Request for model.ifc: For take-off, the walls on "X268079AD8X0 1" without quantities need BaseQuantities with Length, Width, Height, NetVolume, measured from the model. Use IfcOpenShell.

First a look at what the model holds.

```python
import ifcopenshell
import ifcopenshell.util.element
import ifcopenshell.util.unit

model = ifcopenshell.open("model.ifc")
print(model.schema)
for unit_type in ("LENGTHUNIT", "AREAUNIT", "VOLUMEUNIT"):
    print(unit_type, ifcopenshell.util.unit.calculate_unit_scale(model, unit_type))
storey = next(s for s in model.by_type("IfcBuildingStorey") if s.Name == "X268079AD8X0 1")
walls = [e for e in ifcopenshell.util.element.get_decomposition(storey) if e.is_a("IfcWall")]
for e in sorted(walls, key=lambda e: e.id()):
    print(e.id(), e.is_a(), e.Name, list(ifcopenshell.util.element.get_psets(e, qtos_only=True)), sep=" | ")
```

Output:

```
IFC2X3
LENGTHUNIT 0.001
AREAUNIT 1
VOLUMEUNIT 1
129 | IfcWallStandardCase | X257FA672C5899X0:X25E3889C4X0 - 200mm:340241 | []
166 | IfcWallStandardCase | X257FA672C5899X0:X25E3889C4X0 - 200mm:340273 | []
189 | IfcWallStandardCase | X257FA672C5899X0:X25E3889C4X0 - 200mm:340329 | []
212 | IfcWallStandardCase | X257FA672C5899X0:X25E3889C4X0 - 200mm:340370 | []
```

```python
import ifcopenshell
import ifcopenshell.api.pset
import ifcopenshell.geom
import ifcopenshell.util.element
import ifcopenshell.util.shape
import ifcopenshell.util.unit

model = ifcopenshell.open("model.ifc")
unit_scale = ifcopenshell.util.unit.calculate_unit_scale(model)
volume_scale = ifcopenshell.util.unit.calculate_unit_scale(model, "VOLUMEUNIT")
settings = ifcopenshell.geom.settings()

storey = next(s for s in model.by_type("IfcBuildingStorey") if s.Name == "X268079AD8X0 1")
walls = [e for e in ifcopenshell.util.element.get_decomposition(storey) if e.is_a("IfcWall")]

for e in sorted(walls, key=lambda e: e.id()):
    if ifcopenshell.util.element.get_psets(e, qtos_only=True, should_inherit=False):
        continue
    # Geometry comes back in metres, in the element's own axes.
    shape = ifcopenshell.geom.create_shape(settings, e)
    values = {
        "Length": ifcopenshell.util.shape.get_x(shape.geometry) / unit_scale,
        "Width": ifcopenshell.util.shape.get_y(shape.geometry) / unit_scale,
        "Height": ifcopenshell.util.shape.get_z(shape.geometry) / unit_scale,
        "NetVolume": ifcopenshell.util.shape.get_volume(shape.geometry) / volume_scale,
    }
    qto = ifcopenshell.api.pset.add_qto(model, product=e, name="BaseQuantities")
    ifcopenshell.api.pset.edit_qto(model, qto=qto, properties=values)
    print(e.id(), {k: round(v, 3) for k, v in values.items()})

model.write("model-out.ifc")
```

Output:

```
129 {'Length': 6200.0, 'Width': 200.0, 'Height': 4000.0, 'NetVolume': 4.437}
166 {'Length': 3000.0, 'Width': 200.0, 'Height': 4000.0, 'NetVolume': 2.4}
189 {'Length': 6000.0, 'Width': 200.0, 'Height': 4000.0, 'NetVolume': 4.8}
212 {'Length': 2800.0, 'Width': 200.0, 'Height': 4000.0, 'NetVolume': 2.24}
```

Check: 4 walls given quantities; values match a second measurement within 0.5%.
